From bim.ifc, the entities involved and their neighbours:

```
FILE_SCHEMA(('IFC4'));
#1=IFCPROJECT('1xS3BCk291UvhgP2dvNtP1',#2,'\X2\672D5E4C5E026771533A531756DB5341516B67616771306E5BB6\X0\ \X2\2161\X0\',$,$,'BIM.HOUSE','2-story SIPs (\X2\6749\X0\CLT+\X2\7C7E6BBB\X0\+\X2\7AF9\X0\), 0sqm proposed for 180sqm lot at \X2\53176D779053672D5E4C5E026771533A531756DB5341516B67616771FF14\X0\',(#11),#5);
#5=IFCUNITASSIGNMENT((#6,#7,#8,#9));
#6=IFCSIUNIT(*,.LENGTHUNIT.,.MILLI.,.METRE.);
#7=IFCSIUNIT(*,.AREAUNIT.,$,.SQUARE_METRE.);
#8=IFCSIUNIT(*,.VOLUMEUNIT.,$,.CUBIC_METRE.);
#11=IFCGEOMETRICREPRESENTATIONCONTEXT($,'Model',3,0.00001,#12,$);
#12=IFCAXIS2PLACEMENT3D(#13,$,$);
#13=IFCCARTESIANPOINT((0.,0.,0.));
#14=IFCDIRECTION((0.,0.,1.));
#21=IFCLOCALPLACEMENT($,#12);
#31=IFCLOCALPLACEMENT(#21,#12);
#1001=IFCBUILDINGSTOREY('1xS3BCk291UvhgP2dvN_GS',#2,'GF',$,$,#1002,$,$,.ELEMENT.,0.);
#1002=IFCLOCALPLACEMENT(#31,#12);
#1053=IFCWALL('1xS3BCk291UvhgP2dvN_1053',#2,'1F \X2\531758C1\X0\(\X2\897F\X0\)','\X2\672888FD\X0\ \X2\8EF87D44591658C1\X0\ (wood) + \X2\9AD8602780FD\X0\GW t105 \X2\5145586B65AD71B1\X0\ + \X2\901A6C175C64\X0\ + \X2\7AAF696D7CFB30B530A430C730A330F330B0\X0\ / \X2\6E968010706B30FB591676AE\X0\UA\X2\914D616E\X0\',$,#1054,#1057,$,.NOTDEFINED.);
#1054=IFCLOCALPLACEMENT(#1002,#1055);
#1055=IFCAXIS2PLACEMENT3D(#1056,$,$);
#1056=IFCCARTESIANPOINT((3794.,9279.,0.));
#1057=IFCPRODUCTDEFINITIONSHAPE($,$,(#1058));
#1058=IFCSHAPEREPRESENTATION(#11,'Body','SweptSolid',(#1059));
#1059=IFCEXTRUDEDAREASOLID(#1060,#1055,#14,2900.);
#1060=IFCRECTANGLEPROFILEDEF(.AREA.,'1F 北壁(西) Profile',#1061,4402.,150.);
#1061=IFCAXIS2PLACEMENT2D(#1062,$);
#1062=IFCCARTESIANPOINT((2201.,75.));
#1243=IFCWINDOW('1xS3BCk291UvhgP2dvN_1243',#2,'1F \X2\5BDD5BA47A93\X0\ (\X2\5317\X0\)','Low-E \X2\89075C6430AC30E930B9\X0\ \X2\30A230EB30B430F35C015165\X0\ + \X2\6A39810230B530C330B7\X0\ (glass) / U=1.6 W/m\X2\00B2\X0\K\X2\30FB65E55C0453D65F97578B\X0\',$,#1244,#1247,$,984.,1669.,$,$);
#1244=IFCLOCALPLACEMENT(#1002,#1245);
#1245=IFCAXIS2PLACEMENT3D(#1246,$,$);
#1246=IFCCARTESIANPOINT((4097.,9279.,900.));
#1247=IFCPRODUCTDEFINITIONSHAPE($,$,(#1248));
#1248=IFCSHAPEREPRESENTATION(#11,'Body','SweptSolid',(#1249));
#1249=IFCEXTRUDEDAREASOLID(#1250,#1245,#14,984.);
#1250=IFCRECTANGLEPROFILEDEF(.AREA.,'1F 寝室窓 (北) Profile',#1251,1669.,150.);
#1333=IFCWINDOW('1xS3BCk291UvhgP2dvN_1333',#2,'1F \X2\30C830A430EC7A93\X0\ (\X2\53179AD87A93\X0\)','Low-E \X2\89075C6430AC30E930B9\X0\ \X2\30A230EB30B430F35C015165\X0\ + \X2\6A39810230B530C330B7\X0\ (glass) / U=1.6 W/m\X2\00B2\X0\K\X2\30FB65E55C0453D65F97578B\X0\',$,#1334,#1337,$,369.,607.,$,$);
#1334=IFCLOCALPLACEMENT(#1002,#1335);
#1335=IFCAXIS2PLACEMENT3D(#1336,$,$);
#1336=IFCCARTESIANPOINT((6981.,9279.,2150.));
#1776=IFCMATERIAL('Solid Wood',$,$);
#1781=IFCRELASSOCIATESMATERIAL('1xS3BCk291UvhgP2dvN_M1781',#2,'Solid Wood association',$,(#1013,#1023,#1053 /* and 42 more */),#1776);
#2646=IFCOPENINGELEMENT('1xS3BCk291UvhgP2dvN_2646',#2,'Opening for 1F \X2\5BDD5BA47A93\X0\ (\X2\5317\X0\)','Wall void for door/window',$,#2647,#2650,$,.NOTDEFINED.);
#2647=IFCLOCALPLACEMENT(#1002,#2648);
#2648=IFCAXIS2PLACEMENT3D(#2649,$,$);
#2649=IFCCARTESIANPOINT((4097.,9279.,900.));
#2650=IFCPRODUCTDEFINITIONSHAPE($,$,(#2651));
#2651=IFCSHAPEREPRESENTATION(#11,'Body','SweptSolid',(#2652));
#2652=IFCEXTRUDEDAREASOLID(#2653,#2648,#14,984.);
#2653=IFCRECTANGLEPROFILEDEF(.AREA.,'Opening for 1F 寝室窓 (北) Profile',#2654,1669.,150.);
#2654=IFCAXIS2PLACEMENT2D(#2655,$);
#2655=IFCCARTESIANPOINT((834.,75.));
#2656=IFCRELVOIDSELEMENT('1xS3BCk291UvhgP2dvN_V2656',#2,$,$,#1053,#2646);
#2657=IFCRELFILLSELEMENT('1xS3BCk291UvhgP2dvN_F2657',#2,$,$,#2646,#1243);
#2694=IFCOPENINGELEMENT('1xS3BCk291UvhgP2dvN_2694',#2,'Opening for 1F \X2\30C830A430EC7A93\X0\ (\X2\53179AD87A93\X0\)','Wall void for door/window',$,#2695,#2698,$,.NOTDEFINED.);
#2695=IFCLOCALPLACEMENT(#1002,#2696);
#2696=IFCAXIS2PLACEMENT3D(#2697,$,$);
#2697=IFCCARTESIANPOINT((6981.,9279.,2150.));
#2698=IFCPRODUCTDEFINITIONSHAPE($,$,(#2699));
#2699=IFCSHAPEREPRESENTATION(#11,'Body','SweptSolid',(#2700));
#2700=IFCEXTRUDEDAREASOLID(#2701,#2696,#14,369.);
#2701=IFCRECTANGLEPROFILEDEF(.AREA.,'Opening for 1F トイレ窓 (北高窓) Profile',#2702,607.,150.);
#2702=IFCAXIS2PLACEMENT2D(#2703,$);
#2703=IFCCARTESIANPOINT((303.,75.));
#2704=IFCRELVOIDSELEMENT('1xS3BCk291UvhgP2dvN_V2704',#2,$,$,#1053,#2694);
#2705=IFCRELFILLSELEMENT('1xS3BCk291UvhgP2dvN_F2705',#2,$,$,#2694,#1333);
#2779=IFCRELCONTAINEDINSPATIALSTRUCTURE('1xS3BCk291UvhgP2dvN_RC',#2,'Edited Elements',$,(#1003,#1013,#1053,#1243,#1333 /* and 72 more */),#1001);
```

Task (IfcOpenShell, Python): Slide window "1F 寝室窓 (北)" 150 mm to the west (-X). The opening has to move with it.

```python
import ifcopenshell
import ifcopenshell.api.geometry
import ifcopenshell.util.placement

model = ifcopenshell.open("bim.ifc")

window = model.by_guid("1xS3BCk291UvhgP2dvN_1243")
opening = window.FillsVoids[0].RelatingOpeningElement
wall = opening.VoidsElements[0].RelatingBuildingElement

wall_matrix = ifcopenshell.util.placement.get_local_placement(wall.ObjectPlacement)
shift = wall_matrix[:3, 0] * -150.0
before = ifcopenshell.util.placement.get_local_placement(window.ObjectPlacement)[:3, 3].copy()

# The window is not placed relative to its opening, so move both.
for product in (opening, window):
    matrix = ifcopenshell.util.placement.get_local_placement(product.ObjectPlacement)
    matrix[:3, 3] += shift
    ifcopenshell.api.geometry.edit_object_placement(model, product=product, matrix=matrix, is_si=False)

after = ifcopenshell.util.placement.get_local_placement(window.ObjectPlacement)[:3, 3]
print("window moved by", (after - before).round(3) + 0.0)

model.write("bim-out.ifc")
```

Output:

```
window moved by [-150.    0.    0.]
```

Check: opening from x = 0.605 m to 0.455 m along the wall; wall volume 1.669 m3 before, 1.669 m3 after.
